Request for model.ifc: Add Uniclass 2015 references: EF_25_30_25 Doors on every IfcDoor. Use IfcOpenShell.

First a look at what the model holds.

```python
import ifcopenshell

model = ifcopenshell.open("model.ifc")
print(model.schema)
print("classifications:", [c.Name for c in model.by_type("IfcClassification")])
for ifc_class in ("IfcDoor", "IfcRoof", "IfcStair", "IfcWall", "IfcWindow"):
    print(ifc_class, len(model.by_type(ifc_class)))
```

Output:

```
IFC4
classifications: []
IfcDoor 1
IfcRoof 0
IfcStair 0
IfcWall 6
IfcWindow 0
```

```python
import ifcopenshell
import ifcopenshell.api.classification

model = ifcopenshell.open("model.ifc")

system = ifcopenshell.api.classification.add_classification(model, classification="Uniclass 2015")

codes = {
    "IfcDoor": ("EF_25_30_25", "Doors"),
}
for ifc_class, (code, name) in codes.items():
    products = model.by_type(ifc_class)
    ifcopenshell.api.classification.add_reference(
        model, products=products, classification=system, identification=code, name=name
    )
    print(code, len(products))

model.write("model_edited.ifc")
```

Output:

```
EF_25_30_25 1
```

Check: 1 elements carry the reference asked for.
